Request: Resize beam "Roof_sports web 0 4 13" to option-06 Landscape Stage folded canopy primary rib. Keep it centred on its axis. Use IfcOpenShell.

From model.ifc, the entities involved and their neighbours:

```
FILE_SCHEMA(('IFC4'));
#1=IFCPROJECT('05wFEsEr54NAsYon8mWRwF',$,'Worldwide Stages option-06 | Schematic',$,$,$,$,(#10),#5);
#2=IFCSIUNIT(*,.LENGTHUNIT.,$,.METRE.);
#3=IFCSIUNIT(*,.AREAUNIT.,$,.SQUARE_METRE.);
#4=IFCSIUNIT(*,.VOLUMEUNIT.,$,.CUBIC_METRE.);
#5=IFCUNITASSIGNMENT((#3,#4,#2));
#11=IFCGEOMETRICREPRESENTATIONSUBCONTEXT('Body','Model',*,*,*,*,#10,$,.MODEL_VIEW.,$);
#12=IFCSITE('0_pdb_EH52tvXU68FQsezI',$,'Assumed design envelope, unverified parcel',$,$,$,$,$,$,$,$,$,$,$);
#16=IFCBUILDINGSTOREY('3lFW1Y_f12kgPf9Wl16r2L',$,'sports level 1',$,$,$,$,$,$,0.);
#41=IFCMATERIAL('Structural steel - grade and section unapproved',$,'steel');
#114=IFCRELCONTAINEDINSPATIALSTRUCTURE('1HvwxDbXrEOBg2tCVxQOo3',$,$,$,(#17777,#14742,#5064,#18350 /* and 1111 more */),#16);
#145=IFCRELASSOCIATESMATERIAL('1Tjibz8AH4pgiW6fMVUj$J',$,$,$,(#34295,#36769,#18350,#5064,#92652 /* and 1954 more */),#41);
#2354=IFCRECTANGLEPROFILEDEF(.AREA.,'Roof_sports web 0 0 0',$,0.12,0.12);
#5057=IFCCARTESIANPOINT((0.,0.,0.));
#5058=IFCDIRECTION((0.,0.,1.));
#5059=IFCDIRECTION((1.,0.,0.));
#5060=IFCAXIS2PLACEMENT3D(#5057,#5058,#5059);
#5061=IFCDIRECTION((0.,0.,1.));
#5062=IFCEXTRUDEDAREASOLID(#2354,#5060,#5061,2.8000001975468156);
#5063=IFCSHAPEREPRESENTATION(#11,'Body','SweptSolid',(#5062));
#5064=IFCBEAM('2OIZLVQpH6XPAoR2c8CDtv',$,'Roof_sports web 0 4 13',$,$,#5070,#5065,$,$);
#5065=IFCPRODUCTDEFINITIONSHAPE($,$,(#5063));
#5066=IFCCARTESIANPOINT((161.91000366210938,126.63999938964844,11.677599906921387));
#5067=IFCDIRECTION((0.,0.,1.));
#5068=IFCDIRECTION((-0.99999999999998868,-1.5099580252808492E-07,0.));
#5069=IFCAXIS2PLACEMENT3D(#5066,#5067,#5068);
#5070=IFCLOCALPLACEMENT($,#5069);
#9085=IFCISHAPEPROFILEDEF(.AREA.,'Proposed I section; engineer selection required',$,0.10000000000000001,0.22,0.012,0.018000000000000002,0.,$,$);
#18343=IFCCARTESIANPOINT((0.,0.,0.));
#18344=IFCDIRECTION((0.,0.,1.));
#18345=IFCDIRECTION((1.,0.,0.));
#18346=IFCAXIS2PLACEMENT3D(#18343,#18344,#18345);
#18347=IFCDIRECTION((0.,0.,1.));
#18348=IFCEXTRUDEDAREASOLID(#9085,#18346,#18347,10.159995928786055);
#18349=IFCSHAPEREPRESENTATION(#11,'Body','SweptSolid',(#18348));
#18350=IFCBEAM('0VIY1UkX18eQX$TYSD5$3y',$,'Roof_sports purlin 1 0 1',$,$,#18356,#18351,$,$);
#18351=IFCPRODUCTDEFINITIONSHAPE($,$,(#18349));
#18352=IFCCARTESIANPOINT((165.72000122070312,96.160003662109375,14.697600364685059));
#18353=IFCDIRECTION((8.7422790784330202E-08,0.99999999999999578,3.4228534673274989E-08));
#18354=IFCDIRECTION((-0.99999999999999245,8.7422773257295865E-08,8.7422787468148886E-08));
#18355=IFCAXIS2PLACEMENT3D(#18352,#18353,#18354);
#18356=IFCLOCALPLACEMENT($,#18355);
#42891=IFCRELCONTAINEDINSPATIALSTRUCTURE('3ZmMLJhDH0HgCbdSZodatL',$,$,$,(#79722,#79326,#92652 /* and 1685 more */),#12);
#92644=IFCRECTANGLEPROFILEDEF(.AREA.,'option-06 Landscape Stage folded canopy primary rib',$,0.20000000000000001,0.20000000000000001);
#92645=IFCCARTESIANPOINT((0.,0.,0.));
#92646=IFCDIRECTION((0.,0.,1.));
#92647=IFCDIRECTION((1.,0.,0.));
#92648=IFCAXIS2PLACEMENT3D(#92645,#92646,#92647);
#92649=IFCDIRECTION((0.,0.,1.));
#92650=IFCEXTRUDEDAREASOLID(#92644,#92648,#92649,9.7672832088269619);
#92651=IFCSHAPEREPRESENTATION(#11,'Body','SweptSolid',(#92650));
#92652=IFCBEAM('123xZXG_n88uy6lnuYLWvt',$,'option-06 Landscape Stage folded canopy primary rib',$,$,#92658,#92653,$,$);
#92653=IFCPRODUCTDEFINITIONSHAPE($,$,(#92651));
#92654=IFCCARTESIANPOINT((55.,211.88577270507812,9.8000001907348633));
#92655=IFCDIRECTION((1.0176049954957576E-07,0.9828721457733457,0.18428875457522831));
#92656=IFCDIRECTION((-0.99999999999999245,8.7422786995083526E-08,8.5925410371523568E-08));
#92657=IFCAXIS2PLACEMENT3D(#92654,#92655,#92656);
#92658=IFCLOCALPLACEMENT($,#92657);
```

```python
import ifcopenshell
import ifcopenshell.util.element
import ifcopenshell.util.representation

model = ifcopenshell.open("model.ifc")

member = model.by_guid("2OIZLVQpH6XPAoR2c8CDtv")
source = next(p for p in model.by_type("IfcRectangleProfileDef") if p.ProfileName == "option-06 Landscape Stage folded canopy primary rib")

body = ifcopenshell.util.representation.get_representation(member, "Model", "Body")
solid = body.Items[0]
old_profile = solid.SweptArea

# Copy the section's sizes but keep this member's own profile position.
profile = ifcopenshell.util.element.copy(model, source)
profile.Position = old_profile.Position
solid.SweptArea = profile
if not model.get_total_inverses(old_profile):
    ifcopenshell.util.element.remove_deep2(model, old_profile)

print(solid.SweptArea)

model.write("model_rev.ifc")
```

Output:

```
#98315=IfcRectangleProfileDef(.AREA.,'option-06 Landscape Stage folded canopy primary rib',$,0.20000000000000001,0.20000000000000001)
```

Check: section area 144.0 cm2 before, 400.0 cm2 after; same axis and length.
